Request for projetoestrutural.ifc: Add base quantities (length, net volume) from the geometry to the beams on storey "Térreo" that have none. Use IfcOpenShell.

First a look at what the model holds.

```python
import ifcopenshell
import ifcopenshell.util.element
import ifcopenshell.util.unit

model = ifcopenshell.open("projetoestrutural.ifc")
print(model.schema)
for unit_type in ("LENGTHUNIT", "AREAUNIT", "VOLUMEUNIT"):
    print(unit_type, ifcopenshell.util.unit.calculate_unit_scale(model, unit_type))
storey = next(s for s in model.by_type("IfcBuildingStorey") if s.Name == "Térreo")
beams = [e for e in ifcopenshell.util.element.get_decomposition(storey) if e.is_a("IfcBeam")]
for e in sorted(beams, key=lambda e: e.id()):
    print(e.id(), e.is_a(), e.Name, list(ifcopenshell.util.element.get_psets(e, qtos_only=True)), sep=" | ")
```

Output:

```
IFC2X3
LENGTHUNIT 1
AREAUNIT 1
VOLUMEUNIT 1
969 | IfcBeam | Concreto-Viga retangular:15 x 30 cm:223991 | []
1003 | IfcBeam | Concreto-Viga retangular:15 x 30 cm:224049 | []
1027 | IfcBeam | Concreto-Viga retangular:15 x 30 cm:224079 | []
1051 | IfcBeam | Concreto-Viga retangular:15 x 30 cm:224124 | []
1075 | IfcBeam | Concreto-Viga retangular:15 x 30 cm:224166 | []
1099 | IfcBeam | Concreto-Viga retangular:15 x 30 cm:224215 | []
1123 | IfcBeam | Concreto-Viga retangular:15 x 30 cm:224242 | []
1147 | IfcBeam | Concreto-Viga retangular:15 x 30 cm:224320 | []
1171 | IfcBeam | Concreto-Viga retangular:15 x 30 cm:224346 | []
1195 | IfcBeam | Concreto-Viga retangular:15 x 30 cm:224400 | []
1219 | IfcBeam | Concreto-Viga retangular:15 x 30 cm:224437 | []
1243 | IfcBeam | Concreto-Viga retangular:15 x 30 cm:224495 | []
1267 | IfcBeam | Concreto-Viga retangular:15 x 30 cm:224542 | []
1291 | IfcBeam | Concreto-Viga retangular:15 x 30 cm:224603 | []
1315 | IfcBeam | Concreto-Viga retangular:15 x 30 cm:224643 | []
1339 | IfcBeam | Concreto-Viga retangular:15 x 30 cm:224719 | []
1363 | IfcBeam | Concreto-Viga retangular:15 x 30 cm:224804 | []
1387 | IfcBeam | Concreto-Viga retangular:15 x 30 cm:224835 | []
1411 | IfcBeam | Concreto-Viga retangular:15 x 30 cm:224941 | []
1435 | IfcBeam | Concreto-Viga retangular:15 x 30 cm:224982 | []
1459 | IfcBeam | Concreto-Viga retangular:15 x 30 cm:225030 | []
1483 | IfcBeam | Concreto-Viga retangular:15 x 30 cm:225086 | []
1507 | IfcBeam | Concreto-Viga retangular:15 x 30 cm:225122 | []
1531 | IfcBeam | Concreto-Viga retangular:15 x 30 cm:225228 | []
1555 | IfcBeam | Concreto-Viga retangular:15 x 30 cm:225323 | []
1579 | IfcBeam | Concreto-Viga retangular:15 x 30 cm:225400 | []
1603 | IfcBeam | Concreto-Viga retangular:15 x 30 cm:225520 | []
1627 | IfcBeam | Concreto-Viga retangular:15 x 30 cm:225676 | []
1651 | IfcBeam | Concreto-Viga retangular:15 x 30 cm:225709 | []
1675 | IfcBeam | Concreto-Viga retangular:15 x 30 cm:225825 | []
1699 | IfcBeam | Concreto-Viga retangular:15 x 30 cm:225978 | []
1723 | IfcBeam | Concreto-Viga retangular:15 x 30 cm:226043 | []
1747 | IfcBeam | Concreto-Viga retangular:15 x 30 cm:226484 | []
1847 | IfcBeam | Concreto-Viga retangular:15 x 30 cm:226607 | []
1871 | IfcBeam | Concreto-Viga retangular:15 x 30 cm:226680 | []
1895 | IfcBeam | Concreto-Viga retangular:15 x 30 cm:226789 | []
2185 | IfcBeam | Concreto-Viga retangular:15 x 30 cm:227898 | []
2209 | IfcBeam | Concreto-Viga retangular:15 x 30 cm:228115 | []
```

```python
import ifcopenshell
import ifcopenshell.api.pset
import ifcopenshell.geom
import ifcopenshell.util.element
import ifcopenshell.util.shape
import ifcopenshell.util.unit

model = ifcopenshell.open("projetoestrutural.ifc")
unit_scale = ifcopenshell.util.unit.calculate_unit_scale(model)
volume_scale = ifcopenshell.util.unit.calculate_unit_scale(model, "VOLUMEUNIT")
settings = ifcopenshell.geom.settings()

storey = next(s for s in model.by_type("IfcBuildingStorey") if s.Name == "Térreo")
beams = [e for e in ifcopenshell.util.element.get_decomposition(storey) if e.is_a("IfcBeam")]

for e in sorted(beams, key=lambda e: e.id()):
    if ifcopenshell.util.element.get_psets(e, qtos_only=True, should_inherit=False):
        continue
    # Geometry comes back in metres, in the element's own axes.
    shape = ifcopenshell.geom.create_shape(settings, e)
    values = {
        "Length": ifcopenshell.util.shape.get_max_xyz(shape.geometry) / unit_scale,
        "NetVolume": ifcopenshell.util.shape.get_volume(shape.geometry) / volume_scale,
    }
    qto = ifcopenshell.api.pset.add_qto(model, product=e, name="BaseQuantities")
    ifcopenshell.api.pset.edit_qto(model, qto=qto, properties=values)
    print(e.id(), {k: round(v, 3) for k, v in values.items()})

model.write("projetoestrutural_v2.ifc")
```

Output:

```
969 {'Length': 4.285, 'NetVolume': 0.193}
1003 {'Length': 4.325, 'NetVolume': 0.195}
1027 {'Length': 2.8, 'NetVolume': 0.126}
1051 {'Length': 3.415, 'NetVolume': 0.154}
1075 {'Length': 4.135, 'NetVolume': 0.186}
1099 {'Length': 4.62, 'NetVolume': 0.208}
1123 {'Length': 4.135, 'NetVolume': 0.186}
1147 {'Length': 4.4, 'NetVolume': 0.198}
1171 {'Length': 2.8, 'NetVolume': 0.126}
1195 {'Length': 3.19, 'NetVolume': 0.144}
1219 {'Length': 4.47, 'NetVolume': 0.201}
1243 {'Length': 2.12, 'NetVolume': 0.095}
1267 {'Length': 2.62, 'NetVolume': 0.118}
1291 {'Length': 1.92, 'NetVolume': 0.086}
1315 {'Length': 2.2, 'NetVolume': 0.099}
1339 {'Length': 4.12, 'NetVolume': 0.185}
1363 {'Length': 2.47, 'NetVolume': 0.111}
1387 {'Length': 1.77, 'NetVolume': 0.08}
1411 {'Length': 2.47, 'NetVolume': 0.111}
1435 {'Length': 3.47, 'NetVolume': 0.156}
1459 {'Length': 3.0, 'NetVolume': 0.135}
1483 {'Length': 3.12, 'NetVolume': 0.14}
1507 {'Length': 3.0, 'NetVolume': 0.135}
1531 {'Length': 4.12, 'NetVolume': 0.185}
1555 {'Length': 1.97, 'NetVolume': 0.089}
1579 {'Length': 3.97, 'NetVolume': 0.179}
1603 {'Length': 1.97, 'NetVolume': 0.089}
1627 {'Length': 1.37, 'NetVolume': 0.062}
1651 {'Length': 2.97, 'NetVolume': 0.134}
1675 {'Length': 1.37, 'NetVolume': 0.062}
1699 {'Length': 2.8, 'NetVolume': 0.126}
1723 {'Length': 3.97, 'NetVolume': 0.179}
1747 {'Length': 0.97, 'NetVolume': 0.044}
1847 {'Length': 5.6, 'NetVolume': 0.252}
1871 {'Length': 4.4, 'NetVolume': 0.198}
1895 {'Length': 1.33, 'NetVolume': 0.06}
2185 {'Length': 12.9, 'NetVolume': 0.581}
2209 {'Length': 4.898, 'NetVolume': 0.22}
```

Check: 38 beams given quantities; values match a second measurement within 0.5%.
